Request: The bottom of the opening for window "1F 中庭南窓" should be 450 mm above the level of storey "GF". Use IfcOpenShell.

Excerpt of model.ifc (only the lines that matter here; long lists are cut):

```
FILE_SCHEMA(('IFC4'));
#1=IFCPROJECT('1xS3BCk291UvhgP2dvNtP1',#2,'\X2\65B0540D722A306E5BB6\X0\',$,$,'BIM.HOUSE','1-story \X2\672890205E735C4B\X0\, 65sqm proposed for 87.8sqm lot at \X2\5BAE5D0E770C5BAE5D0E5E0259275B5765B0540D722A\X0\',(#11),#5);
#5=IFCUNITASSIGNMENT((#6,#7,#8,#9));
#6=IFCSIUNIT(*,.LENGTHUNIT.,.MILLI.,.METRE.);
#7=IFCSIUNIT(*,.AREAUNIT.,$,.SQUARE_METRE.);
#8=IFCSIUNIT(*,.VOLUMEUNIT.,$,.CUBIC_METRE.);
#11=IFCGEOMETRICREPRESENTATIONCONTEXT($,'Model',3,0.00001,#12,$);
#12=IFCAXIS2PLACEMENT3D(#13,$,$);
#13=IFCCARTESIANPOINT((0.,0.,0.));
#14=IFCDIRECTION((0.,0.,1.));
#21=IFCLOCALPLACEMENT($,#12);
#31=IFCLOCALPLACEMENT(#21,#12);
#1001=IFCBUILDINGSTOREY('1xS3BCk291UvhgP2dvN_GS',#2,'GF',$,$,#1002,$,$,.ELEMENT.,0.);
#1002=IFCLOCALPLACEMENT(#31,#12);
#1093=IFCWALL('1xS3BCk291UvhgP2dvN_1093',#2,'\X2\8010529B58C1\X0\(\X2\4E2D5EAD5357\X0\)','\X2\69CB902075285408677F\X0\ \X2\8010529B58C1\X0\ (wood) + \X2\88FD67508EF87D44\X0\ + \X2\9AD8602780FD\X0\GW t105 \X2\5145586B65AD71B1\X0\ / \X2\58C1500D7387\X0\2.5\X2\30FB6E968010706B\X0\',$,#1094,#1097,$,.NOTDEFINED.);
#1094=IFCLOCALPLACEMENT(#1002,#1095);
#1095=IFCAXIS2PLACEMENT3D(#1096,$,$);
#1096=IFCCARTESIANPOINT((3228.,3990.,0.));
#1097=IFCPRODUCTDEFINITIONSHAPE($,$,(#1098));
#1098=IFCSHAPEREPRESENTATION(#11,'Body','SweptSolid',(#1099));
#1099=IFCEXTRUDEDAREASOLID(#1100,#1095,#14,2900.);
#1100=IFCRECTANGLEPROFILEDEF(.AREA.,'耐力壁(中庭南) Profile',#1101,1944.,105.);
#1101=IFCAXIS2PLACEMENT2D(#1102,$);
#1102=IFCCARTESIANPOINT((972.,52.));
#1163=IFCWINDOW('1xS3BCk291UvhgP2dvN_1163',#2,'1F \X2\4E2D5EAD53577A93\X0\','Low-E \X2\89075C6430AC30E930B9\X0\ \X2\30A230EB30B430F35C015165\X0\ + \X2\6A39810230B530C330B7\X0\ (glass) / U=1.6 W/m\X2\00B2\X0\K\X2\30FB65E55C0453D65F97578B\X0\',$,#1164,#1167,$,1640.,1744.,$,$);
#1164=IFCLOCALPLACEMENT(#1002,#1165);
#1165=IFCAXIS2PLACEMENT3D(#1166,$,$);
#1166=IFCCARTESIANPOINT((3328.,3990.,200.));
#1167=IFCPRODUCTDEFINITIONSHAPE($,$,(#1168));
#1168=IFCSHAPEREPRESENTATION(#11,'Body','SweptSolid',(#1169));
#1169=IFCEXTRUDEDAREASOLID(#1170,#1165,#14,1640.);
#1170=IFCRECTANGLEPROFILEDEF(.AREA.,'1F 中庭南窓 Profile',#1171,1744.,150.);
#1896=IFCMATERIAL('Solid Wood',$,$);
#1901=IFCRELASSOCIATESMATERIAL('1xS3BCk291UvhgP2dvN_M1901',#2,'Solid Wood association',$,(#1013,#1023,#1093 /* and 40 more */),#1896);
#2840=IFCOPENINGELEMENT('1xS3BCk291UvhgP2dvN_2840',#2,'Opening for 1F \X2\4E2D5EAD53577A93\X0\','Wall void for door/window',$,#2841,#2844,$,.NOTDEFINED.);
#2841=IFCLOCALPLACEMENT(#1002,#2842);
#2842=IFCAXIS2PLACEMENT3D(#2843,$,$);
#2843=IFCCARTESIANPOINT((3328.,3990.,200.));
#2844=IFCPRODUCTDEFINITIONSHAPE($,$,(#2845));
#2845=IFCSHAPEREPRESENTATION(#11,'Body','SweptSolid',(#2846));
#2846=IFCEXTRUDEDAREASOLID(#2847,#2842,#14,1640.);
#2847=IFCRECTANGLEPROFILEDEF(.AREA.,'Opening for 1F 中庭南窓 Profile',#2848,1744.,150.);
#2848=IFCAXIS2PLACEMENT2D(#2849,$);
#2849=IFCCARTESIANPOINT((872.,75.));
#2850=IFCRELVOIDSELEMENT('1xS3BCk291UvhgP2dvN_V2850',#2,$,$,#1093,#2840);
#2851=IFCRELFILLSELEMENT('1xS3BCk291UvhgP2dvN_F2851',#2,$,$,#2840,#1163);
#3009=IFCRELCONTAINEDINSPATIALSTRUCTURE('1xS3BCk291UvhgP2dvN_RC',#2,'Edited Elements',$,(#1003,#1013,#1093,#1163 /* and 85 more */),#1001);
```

```python
import numpy as np
import ifcopenshell
import ifcopenshell.api.geometry
import ifcopenshell.geom
import ifcopenshell.util.element
import ifcopenshell.util.placement
import ifcopenshell.util.shape
import ifcopenshell.util.unit

model = ifcopenshell.open("model.ifc")
unit_scale = ifcopenshell.util.unit.calculate_unit_scale(model)

window = model.by_guid("1xS3BCk291UvhgP2dvN_1163")
opening = window.FillsVoids[0].RelatingOpeningElement
storey = ifcopenshell.util.element.get_container(window, ifc_class="IfcBuildingStorey")
level = ifcopenshell.util.placement.get_local_placement(storey.ObjectPlacement)[2, 3]

# The opening's origin need not be at the sill, so measure its lowest point.
shape = ifcopenshell.geom.create_shape(ifcopenshell.geom.settings(), opening)
bottom = ifcopenshell.util.shape.get_shape_bottom_elevation(shape, shape.geometry) / unit_scale
dz = level + 450.0 - bottom

shift = np.array([0.0, 0.0, dz])
# The window is not placed relative to its opening, so move both.
for product in (opening, window):
    matrix = ifcopenshell.util.placement.get_local_placement(product.ObjectPlacement)
    matrix[:3, 3] += shift
    ifcopenshell.api.geometry.edit_object_placement(model, product=product, matrix=matrix, is_si=False)

print(f"moved by {dz * unit_scale:+.3f} m")

model.write("model_rev.ifc")
```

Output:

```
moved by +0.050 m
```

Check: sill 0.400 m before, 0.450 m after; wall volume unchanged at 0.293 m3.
